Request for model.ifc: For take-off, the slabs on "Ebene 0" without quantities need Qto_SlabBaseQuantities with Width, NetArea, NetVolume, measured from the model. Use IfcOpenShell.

First a look at what the model holds.

```python
import ifcopenshell
import ifcopenshell.util.element
import ifcopenshell.util.unit

model = ifcopenshell.open("model.ifc")
print(model.schema)
for unit_type in ("LENGTHUNIT", "AREAUNIT", "VOLUMEUNIT"):
    print(unit_type, ifcopenshell.util.unit.calculate_unit_scale(model, unit_type))
storey = next(s for s in model.by_type("IfcBuildingStorey") if s.Name == "Ebene 0")
slabs = [e for e in ifcopenshell.util.element.get_decomposition(storey) if e.is_a("IfcSlab")]
for e in sorted(slabs, key=lambda e: e.id()):
    print(e.id(), e.is_a(), e.Name, list(ifcopenshell.util.element.get_psets(e, qtos_only=True)), sep=" | ")
```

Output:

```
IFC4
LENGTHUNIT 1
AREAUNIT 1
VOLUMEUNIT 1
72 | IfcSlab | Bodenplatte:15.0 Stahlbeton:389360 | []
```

```python
import ifcopenshell
import ifcopenshell.api.pset
import ifcopenshell.geom
import ifcopenshell.util.element
import ifcopenshell.util.shape
import ifcopenshell.util.unit

model = ifcopenshell.open("model.ifc")
unit_scale = ifcopenshell.util.unit.calculate_unit_scale(model)
area_scale = ifcopenshell.util.unit.calculate_unit_scale(model, "AREAUNIT")
volume_scale = ifcopenshell.util.unit.calculate_unit_scale(model, "VOLUMEUNIT")
settings = ifcopenshell.geom.settings()

storey = next(s for s in model.by_type("IfcBuildingStorey") if s.Name == "Ebene 0")
slabs = [e for e in ifcopenshell.util.element.get_decomposition(storey) if e.is_a("IfcSlab")]

for e in sorted(slabs, key=lambda e: e.id()):
    if ifcopenshell.util.element.get_psets(e, qtos_only=True, should_inherit=False):
        continue
    # Geometry comes back in metres, in the element's own axes.
    shape = ifcopenshell.geom.create_shape(settings, e)
    values = {
        "Width": ifcopenshell.util.shape.get_z(shape.geometry) / unit_scale,
        "NetArea": ifcopenshell.util.shape.get_footprint_area(shape.geometry) / area_scale,
        "NetVolume": ifcopenshell.util.shape.get_volume(shape.geometry) / volume_scale,
    }
    qto = ifcopenshell.api.pset.add_qto(model, product=e, name="Qto_SlabBaseQuantities")
    ifcopenshell.api.pset.edit_qto(model, qto=qto, properties=values)
    print(e.id(), {k: round(v, 3) for k, v in values.items()})

model.write("model_updated.ifc")
```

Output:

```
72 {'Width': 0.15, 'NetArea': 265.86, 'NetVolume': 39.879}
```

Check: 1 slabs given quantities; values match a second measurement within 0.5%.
